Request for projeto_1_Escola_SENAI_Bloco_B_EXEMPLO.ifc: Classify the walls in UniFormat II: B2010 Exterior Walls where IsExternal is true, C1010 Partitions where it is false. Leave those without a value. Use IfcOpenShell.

First a look at what the model holds.

```python
import ifcopenshell
import ifcopenshell.util.element

model = ifcopenshell.open("projeto_1_Escola_SENAI_Bloco_B_EXEMPLO.ifc")
print(model.schema)
print("classifications:", [c.Name for c in model.by_type("IfcClassification")])
values = [ifcopenshell.util.element.get_pset(e, "Pset_WallCommon", "IsExternal") for e in model.by_type("IfcWall")]
for value in (True, False, None):
    print("IsExternal", value, values.count(value))
```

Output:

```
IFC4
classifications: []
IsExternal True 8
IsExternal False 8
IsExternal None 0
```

```python
import ifcopenshell
import ifcopenshell.api.classification
import ifcopenshell.util.element

model = ifcopenshell.open("projeto_1_Escola_SENAI_Bloco_B_EXEMPLO.ifc")

system = ifcopenshell.api.classification.add_classification(model, classification="UniFormat II")

walls = model.by_type("IfcWall")
external = {e: ifcopenshell.util.element.get_pset(e, "Pset_WallCommon", "IsExternal") for e in walls}
for flag, code, name in ((True, "B2010", "Exterior Walls"), (False, "C1010", "Partitions")):
    products = [e for e in walls if external[e] is flag]
    ifcopenshell.api.classification.add_reference(
        model, products=products, classification=system, identification=code, name=name
    )
    print(code, len(products))

model.write("projeto_1_Escola_SENAI_Bloco_B_EXEMPLO-out.ifc")
```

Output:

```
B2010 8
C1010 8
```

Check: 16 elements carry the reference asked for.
